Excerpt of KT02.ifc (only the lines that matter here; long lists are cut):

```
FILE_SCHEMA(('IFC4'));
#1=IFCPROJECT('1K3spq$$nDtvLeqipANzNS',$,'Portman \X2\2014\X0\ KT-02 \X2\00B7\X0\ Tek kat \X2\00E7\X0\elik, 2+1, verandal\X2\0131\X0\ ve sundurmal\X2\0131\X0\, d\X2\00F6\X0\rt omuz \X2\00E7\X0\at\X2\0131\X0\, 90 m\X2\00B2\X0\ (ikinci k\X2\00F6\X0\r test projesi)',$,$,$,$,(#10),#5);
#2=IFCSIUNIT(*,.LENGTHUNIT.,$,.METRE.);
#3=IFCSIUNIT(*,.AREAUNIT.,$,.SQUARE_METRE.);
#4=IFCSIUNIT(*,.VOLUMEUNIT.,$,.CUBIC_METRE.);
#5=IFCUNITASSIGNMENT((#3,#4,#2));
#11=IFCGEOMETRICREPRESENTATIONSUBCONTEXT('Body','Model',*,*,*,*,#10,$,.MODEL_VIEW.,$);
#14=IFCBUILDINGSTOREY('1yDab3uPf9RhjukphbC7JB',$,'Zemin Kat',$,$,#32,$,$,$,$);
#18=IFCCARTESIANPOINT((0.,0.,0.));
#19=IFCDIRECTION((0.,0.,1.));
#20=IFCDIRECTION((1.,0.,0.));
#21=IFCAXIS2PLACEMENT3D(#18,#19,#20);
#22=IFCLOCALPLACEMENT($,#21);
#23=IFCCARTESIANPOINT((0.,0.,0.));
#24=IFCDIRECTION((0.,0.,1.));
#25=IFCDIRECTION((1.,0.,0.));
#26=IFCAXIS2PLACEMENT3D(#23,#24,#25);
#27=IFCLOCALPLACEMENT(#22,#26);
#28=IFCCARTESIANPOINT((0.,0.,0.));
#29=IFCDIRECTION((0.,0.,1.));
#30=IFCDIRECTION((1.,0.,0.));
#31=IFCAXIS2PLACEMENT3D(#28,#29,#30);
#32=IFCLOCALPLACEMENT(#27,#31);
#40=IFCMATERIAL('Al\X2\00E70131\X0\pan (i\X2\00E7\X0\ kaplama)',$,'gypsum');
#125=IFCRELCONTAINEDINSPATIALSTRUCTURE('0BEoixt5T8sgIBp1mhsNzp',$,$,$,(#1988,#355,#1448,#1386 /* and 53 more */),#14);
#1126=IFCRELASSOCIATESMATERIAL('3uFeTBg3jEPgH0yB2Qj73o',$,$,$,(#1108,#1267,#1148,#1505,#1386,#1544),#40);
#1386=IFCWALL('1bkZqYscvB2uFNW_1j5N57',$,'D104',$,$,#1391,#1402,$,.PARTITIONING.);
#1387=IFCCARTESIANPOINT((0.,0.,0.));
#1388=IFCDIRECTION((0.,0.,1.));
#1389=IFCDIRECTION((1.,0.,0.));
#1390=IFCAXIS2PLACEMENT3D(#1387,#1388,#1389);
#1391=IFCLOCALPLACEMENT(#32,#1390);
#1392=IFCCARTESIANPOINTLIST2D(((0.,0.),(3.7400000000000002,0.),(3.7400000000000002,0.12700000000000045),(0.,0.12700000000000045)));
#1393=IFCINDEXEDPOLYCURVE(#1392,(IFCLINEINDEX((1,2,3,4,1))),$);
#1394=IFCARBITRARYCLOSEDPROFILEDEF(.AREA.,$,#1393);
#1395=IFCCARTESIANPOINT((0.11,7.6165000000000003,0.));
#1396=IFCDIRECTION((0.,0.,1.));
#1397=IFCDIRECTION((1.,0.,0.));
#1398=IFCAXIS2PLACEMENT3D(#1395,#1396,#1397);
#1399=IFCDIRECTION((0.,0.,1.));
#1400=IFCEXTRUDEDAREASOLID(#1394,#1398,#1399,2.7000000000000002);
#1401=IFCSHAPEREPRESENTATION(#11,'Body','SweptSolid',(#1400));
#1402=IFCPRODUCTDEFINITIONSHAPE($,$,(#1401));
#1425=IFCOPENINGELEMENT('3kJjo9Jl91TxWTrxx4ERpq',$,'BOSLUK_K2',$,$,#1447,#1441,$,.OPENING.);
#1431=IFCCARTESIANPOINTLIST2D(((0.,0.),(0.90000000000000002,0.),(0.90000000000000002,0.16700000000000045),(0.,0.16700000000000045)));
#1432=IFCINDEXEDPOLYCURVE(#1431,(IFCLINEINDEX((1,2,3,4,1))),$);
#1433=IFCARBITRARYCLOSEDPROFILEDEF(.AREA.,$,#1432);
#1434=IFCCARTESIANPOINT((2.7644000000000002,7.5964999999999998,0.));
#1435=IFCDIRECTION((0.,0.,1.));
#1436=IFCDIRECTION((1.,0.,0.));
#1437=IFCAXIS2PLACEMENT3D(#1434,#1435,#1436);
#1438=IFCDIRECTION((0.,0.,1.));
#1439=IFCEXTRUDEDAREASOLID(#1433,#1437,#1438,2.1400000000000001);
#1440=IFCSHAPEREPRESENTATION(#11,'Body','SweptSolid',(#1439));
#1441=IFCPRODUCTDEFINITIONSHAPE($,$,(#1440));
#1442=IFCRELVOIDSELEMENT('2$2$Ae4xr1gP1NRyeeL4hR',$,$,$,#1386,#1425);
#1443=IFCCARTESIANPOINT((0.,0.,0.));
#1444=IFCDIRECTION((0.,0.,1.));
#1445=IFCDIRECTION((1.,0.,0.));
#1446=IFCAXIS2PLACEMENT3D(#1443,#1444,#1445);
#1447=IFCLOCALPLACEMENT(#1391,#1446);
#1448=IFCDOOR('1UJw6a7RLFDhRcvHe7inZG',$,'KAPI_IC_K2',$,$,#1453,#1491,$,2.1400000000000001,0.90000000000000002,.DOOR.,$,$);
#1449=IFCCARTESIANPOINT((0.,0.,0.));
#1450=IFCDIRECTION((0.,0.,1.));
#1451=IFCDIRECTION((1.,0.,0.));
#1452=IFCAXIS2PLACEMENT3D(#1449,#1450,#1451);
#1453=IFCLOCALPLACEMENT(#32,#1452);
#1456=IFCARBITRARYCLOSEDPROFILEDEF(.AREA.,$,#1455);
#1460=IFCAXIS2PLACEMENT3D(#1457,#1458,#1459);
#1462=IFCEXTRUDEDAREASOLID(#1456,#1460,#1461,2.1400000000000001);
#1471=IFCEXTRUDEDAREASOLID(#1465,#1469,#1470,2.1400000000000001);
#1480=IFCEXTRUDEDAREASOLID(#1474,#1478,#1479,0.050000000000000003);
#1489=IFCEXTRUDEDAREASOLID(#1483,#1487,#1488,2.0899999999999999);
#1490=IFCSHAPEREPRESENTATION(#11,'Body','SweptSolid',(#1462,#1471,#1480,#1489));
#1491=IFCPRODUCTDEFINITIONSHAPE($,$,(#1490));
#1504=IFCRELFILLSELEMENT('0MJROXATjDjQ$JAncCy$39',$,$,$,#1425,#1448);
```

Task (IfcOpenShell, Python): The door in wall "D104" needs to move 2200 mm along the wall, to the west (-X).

```python
import ifcopenshell
import ifcopenshell.api.geometry
import ifcopenshell.util.placement
import ifcopenshell.util.unit

model = ifcopenshell.open("KT02.ifc")
unit_scale = ifcopenshell.util.unit.calculate_unit_scale(model)

door = model.by_guid("1UJw6a7RLFDhRcvHe7inZG")
opening = door.FillsVoids[0].RelatingOpeningElement
wall = opening.VoidsElements[0].RelatingBuildingElement

wall_matrix = ifcopenshell.util.placement.get_local_placement(wall.ObjectPlacement)
shift = wall_matrix[:3, 0] * -2.2 / unit_scale
before = ifcopenshell.util.placement.get_local_placement(door.ObjectPlacement)[:3, 3].copy()

# The door is not placed relative to its opening, so move both.
for product in (opening, door):
    matrix = ifcopenshell.util.placement.get_local_placement(product.ObjectPlacement)
    matrix[:3, 3] += shift
    ifcopenshell.api.geometry.edit_object_placement(model, product=product, matrix=matrix, is_si=False)

after = ifcopenshell.util.placement.get_local_placement(door.ObjectPlacement)[:3, 3]
print("door moved by", (after - before).round(3) + 0.0)

model.write("KT02_updated.ifc")
```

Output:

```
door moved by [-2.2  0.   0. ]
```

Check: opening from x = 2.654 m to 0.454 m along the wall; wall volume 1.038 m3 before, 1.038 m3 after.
